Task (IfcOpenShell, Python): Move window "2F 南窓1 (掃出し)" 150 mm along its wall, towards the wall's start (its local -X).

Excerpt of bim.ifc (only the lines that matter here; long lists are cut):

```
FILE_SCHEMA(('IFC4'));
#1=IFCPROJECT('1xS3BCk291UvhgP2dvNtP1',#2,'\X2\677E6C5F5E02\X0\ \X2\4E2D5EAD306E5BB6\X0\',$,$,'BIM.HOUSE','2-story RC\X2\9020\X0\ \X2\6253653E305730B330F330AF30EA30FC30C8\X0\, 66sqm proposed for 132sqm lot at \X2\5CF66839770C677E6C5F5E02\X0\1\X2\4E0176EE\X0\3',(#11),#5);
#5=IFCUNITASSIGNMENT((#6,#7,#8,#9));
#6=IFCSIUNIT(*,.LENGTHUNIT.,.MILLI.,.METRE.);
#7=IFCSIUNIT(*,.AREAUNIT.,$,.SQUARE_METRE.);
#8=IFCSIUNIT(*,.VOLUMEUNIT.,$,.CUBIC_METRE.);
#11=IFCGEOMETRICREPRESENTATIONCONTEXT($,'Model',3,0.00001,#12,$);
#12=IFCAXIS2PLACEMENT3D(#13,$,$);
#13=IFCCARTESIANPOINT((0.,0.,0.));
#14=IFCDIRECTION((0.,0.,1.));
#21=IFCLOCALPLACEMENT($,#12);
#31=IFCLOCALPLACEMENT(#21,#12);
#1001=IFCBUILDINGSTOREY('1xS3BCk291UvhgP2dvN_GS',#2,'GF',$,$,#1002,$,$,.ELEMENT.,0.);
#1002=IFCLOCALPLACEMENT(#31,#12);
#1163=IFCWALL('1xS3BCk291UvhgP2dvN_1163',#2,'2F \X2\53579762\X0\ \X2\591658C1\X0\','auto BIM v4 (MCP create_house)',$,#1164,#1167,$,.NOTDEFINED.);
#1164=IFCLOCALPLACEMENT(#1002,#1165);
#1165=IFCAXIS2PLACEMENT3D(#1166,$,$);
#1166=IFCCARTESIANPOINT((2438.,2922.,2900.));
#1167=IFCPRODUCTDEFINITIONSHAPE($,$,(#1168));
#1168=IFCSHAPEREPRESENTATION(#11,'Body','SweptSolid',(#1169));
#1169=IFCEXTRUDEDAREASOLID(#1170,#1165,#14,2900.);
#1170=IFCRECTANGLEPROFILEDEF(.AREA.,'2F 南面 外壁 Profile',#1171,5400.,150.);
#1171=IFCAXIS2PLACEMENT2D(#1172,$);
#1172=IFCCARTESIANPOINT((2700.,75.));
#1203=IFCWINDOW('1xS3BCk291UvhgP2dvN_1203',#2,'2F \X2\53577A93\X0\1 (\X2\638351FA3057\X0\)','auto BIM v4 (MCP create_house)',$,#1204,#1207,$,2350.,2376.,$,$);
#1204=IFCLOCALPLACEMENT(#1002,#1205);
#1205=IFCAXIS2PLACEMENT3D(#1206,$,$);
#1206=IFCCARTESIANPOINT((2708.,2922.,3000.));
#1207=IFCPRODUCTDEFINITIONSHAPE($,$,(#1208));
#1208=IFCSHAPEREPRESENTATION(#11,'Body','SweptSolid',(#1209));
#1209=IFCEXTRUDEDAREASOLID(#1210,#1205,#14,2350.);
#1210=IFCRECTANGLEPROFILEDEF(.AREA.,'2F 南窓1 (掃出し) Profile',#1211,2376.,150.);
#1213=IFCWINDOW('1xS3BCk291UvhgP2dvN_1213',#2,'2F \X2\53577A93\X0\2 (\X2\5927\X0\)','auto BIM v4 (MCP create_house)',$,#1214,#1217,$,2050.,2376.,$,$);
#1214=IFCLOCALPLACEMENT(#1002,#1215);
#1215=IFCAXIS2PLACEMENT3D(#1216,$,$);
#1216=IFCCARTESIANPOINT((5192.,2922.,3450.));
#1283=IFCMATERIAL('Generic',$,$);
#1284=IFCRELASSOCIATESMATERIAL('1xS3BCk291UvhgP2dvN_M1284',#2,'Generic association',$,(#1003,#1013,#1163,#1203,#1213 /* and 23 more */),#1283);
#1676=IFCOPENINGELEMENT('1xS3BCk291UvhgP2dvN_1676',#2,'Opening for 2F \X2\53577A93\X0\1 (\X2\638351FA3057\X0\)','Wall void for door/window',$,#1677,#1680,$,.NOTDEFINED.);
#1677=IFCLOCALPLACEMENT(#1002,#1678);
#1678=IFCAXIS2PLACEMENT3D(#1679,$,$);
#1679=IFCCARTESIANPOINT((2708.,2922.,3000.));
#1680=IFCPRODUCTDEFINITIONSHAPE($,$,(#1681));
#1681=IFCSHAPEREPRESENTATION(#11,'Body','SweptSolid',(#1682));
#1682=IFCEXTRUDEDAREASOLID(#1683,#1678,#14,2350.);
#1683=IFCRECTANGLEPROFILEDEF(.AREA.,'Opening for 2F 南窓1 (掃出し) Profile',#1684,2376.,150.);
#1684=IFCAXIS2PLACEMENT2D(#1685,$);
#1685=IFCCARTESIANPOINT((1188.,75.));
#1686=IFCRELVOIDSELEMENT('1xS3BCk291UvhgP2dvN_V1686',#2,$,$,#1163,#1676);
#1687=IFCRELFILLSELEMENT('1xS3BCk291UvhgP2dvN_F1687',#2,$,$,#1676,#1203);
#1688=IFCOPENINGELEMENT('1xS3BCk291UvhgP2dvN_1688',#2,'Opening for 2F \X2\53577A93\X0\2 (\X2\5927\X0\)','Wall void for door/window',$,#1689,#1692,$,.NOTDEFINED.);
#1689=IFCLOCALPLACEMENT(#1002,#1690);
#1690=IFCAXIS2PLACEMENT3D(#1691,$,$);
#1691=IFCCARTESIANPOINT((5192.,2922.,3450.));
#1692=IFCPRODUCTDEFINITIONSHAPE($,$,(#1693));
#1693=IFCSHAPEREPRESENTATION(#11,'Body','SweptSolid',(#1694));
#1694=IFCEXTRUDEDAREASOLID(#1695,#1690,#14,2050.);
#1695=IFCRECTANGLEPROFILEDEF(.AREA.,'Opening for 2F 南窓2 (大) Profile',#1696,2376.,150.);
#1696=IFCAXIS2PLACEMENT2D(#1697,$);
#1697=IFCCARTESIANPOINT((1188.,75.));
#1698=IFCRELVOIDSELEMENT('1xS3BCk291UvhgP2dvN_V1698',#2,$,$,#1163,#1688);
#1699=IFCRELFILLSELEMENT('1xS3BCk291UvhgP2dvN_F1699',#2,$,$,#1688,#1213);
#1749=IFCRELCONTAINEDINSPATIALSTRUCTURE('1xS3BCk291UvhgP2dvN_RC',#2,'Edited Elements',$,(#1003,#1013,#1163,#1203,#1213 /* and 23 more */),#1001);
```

```python
import ifcopenshell
import ifcopenshell.api.geometry
import ifcopenshell.util.placement

model = ifcopenshell.open("bim.ifc")

window = model.by_guid("1xS3BCk291UvhgP2dvN_1203")
opening = window.FillsVoids[0].RelatingOpeningElement
wall = opening.VoidsElements[0].RelatingBuildingElement

wall_matrix = ifcopenshell.util.placement.get_local_placement(wall.ObjectPlacement)
shift = wall_matrix[:3, 0] * -150.0
before = ifcopenshell.util.placement.get_local_placement(window.ObjectPlacement)[:3, 3].copy()

# The window is not placed relative to its opening, so move both.
for product in (opening, window):
    matrix = ifcopenshell.util.placement.get_local_placement(product.ObjectPlacement)
    matrix[:3, 3] += shift
    ifcopenshell.api.geometry.edit_object_placement(model, product=product, matrix=matrix, is_si=False)

after = ifcopenshell.util.placement.get_local_placement(window.ObjectPlacement)[:3, 3]
print("window moved by", (after - before).round(3) + 0.0)

model.write("bim_edited.ifc")
```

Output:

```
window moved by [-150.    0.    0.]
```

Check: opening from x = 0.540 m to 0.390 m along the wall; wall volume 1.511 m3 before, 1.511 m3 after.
